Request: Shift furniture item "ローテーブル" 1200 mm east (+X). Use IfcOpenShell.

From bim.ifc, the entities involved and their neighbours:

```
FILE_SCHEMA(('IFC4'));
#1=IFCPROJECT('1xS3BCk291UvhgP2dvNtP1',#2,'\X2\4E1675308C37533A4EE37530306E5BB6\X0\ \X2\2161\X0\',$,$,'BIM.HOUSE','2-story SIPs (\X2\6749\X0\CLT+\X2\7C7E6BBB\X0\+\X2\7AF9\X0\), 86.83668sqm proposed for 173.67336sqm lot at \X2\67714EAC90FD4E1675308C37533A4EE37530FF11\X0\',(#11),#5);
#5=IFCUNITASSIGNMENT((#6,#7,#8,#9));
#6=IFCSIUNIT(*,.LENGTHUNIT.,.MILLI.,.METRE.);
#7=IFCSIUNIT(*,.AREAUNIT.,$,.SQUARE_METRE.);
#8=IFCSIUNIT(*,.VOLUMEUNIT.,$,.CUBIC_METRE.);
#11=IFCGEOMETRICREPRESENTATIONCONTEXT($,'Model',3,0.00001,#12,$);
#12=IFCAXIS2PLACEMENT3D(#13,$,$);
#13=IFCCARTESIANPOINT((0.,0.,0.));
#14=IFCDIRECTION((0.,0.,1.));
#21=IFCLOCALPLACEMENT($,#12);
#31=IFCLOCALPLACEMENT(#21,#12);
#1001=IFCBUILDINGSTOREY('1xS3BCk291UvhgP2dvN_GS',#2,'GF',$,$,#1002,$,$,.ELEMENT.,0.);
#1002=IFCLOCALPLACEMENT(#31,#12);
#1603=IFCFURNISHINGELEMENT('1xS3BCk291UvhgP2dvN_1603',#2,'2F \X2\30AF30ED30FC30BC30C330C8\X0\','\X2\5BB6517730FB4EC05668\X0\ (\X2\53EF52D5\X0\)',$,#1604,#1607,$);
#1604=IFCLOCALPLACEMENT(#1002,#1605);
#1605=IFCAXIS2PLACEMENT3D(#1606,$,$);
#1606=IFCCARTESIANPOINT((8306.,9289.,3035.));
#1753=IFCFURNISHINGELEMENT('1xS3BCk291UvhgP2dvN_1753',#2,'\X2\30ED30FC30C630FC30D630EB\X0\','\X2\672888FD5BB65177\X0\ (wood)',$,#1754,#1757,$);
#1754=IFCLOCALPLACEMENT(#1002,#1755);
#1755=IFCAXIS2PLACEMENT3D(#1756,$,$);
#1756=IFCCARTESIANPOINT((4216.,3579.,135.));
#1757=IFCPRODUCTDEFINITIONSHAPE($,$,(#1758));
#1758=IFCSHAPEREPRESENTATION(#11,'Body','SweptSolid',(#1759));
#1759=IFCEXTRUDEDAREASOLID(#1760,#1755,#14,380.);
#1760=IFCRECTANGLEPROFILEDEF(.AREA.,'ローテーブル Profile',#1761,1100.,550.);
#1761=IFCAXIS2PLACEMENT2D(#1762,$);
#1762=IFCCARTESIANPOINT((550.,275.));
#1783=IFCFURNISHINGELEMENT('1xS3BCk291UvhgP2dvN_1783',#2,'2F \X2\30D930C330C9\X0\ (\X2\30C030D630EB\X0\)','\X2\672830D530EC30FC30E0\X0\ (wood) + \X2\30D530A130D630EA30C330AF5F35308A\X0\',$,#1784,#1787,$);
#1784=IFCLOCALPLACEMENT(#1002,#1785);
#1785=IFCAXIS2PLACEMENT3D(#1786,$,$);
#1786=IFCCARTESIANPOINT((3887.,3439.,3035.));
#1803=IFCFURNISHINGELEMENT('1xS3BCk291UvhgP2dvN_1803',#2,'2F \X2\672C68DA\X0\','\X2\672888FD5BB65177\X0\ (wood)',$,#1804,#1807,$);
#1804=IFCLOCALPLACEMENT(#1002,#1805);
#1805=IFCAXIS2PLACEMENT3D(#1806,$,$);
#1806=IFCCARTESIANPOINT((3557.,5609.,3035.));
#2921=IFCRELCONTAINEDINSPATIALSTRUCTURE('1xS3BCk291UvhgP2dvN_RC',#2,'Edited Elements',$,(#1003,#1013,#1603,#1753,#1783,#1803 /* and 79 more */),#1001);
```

```python
import ifcopenshell
import ifcopenshell.api.geometry
import ifcopenshell.util.placement
import ifcopenshell.util.unit

model = ifcopenshell.open("bim.ifc")
unit_scale = ifcopenshell.util.unit.calculate_unit_scale(model)

item = model.by_id(1753)
matrix = ifcopenshell.util.placement.get_local_placement(item.ObjectPlacement)
matrix[0, 3] += 1.2 / unit_scale
ifcopenshell.api.geometry.edit_object_placement(model, product=item, matrix=matrix, is_si=False)

print(ifcopenshell.util.placement.get_local_placement(item.ObjectPlacement).round(3) + 0.0)

model.write("bim_updated.ifc")
```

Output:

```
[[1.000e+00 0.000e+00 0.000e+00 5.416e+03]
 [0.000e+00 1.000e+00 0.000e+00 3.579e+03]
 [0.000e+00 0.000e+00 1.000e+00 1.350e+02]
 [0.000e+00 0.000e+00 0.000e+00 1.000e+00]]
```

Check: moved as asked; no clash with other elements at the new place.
